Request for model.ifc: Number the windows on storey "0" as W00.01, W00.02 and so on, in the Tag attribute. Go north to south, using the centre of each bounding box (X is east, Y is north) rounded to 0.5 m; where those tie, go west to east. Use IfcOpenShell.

First a look at what the model holds.

```python
import ifcopenshell
import ifcopenshell.util.element
import ifcopenshell.util.placement

model = ifcopenshell.open("model.ifc")
print(model.schema)
storey = next(s for s in model.by_type("IfcBuildingStorey") if s.Name == "0")
windows = [e for e in ifcopenshell.util.element.get_decomposition(storey) if e.is_a("IfcWindow")]
for e in sorted(windows, key=lambda e: e.id()):
    origin = ifcopenshell.util.placement.get_local_placement(e.ObjectPlacement)[:3, 3]
    print(e.id(), e.Tag, e.Name, origin.round(2) + 0.0, sep=" | ")
```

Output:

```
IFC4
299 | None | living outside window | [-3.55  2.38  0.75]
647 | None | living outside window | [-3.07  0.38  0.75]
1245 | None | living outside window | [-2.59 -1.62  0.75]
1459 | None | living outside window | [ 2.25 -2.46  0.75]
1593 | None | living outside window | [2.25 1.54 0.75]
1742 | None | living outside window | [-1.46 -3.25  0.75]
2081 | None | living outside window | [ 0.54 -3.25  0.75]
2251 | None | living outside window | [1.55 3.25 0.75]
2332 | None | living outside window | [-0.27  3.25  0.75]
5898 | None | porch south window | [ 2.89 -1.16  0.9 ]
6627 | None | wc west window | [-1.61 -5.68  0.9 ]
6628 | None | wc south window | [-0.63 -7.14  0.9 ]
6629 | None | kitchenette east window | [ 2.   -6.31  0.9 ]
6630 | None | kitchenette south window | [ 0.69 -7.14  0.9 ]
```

```python
import ifcopenshell
import ifcopenshell.geom
import ifcopenshell.util.element
import ifcopenshell.util.shape

model = ifcopenshell.open("model.ifc")
settings = ifcopenshell.geom.settings()
settings.set("use-world-coords", True)


def centre(element):
    shape = ifcopenshell.geom.create_shape(settings, element)
    return ifcopenshell.util.shape.get_bbox_centroid(shape.geometry)


storey = next(s for s in model.by_type("IfcBuildingStorey") if s.Name == "0")
windows = [e for e in ifcopenshell.util.element.get_decomposition(storey) if e.is_a("IfcWindow")]

# Insertion points can sit at a corner or the storey origin, so sort by the geometry (in metres).
centres = {e: centre(e) for e in windows}
windows.sort(key=lambda e: (-round(centres[e][1] / 0.5), centres[e][0]))

for i, e in enumerate(windows, start=1):
    number = f"W00.{i:02d}"
    e.Tag = number
    print(e.id(), number)

model.write("model_updated.ifc")
```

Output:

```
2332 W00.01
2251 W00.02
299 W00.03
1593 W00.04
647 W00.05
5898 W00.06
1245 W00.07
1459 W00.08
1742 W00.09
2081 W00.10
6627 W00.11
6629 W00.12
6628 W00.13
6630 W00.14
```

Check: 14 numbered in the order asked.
